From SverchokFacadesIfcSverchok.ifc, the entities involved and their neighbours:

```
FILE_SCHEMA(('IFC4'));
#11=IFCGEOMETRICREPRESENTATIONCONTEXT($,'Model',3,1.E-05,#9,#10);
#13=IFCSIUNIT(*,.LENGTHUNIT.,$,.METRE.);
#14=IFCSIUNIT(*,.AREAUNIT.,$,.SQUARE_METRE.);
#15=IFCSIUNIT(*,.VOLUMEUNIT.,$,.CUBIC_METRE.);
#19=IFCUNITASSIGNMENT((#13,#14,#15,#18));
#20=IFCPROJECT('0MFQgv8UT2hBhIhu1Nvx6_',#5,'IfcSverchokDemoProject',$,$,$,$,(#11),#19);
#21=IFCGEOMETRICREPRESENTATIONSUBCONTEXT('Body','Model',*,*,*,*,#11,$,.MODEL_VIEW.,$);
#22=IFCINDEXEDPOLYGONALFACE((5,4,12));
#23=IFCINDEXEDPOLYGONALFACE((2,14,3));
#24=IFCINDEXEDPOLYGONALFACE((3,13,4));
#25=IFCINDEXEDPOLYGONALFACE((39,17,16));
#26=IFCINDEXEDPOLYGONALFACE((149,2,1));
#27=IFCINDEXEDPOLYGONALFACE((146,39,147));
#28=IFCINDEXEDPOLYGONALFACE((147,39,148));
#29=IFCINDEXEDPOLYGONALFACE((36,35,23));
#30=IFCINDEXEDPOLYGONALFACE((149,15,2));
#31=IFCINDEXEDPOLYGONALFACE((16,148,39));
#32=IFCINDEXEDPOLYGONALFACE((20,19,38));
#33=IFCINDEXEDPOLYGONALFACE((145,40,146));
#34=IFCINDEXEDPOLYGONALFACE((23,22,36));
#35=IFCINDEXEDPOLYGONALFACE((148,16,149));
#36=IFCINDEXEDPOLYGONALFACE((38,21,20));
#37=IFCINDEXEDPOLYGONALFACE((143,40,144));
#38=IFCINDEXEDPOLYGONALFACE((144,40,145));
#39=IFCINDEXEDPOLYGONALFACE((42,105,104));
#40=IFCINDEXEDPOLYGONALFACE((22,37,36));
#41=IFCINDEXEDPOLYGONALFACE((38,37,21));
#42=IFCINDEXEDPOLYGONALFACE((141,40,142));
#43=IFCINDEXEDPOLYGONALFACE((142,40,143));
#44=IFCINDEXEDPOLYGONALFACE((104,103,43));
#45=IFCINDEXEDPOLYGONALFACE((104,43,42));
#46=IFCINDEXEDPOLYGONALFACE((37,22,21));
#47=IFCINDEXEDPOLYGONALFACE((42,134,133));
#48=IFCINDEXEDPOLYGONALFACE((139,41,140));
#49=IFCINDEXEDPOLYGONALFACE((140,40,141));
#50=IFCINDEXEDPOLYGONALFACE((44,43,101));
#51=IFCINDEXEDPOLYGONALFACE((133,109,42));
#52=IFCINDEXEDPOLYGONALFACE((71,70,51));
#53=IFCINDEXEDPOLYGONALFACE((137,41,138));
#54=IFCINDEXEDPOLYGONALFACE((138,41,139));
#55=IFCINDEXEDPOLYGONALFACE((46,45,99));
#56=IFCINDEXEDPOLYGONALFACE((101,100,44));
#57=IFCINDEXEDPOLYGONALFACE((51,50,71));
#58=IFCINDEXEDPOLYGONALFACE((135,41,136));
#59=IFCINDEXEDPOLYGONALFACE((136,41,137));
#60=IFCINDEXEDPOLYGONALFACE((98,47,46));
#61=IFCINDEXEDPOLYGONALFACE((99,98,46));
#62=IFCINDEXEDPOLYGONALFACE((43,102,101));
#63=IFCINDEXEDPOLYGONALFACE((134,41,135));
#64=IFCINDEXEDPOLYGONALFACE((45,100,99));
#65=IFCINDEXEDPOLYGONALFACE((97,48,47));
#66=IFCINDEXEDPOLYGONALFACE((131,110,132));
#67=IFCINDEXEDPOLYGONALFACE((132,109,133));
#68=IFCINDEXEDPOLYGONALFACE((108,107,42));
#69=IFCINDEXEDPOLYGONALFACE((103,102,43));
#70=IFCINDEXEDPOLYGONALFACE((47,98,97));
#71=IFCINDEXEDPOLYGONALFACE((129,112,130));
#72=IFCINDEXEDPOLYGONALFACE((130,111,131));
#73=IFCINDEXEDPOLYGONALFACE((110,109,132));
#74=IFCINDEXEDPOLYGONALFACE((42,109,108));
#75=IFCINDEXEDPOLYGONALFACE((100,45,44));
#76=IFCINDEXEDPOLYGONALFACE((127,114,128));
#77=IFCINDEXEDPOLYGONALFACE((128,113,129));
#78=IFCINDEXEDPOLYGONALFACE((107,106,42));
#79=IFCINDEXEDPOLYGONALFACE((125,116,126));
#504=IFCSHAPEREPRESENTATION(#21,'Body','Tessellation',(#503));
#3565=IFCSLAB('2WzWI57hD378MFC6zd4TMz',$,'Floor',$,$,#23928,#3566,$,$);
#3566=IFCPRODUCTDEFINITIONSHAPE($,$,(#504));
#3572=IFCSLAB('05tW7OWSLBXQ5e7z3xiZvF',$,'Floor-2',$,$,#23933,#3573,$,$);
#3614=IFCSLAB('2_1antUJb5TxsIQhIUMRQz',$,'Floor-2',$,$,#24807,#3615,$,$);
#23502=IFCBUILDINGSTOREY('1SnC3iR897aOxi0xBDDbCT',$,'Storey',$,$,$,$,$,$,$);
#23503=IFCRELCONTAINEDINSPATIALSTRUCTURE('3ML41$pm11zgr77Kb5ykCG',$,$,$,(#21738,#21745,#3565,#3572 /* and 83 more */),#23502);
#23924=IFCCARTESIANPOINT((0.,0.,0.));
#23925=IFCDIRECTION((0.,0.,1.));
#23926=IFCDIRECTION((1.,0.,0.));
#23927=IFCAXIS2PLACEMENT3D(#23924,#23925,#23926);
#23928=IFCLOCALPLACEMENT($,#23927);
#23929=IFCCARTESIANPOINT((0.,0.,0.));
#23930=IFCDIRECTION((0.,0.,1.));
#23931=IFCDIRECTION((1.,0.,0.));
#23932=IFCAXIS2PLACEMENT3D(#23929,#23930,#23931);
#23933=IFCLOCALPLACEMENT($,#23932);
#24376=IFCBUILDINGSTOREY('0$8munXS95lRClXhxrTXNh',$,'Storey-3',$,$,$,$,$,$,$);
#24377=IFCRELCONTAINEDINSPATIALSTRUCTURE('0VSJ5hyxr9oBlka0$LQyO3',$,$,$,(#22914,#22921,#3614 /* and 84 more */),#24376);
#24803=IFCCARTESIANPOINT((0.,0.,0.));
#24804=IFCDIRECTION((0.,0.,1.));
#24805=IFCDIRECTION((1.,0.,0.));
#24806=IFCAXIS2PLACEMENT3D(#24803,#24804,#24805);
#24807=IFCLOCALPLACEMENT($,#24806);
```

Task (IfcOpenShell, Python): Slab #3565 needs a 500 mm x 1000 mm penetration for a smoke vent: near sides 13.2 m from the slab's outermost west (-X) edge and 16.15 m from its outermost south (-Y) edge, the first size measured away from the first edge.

```python
import numpy as np
import ifcopenshell
import ifcopenshell.api.feature
import ifcopenshell.api.geometry
import ifcopenshell.api.root
import ifcopenshell.geom
import ifcopenshell.util.placement
import ifcopenshell.util.representation
import ifcopenshell.util.shape
import ifcopenshell.util.unit

model = ifcopenshell.open("SverchokFacadesIfcSverchok.ifc")
unit_scale = ifcopenshell.util.unit.calculate_unit_scale(model)
settings = ifcopenshell.geom.settings()


def volume(element):
    """Net volume in cubic metres, openings subtracted."""
    shape = ifcopenshell.geom.create_shape(settings, element)
    return ifcopenshell.util.shape.get_volume(shape.geometry)


slab = model.by_guid("2WzWI57hD378MFC6zd4TMz")
before = volume(slab)

# Extent in the slab's own axes, in metres. The edges named are its -X and -Y sides.
slab_shape = ifcopenshell.geom.create_shape(settings, slab)
vertices = ifcopenshell.util.shape.get_vertices(slab_shape.geometry)
x_min, y_min, bottom = vertices.min(axis=0)
top = vertices[:, 2].max()

opening = ifcopenshell.api.root.create_entity(model, ifc_class="IfcOpeningElement", name="Smoke vent opening", predefined_type="OPENING")
context = ifcopenshell.util.representation.get_context(model, "Model", "Body", "MODEL_VIEW")
width, depth = 0.5, 1
outline = [(0.0, 0.0), (width, 0.0), (width, depth), (0.0, depth), (0.0, 0.0)]
# Overshoot both faces by 50 mm so the cut is clean.
shape = ifcopenshell.api.geometry.add_slab_representation(
    model, context=context, depth=top - bottom + 0.1, polyline=outline
)
ifcopenshell.api.geometry.assign_representation(model, product=opening, representation=shape)

matrix = ifcopenshell.util.placement.get_local_placement(slab.ObjectPlacement)
matrix[:, 3] = matrix @ np.append(np.array([x_min + 13.2, y_min + 16.15, bottom - 0.05]) / unit_scale, 1.0)
ifcopenshell.api.geometry.edit_object_placement(model, product=opening, matrix=matrix, is_si=False)
ifcopenshell.api.feature.add_feature(model, feature=opening, element=slab)

after = volume(slab)

print(f"slab volume {before:.3f} -> {after:.3f} m3")

model.write("SverchokFacadesIfcSverchok_v2.ifc")
```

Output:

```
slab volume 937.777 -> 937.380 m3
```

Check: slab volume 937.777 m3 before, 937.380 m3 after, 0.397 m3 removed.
